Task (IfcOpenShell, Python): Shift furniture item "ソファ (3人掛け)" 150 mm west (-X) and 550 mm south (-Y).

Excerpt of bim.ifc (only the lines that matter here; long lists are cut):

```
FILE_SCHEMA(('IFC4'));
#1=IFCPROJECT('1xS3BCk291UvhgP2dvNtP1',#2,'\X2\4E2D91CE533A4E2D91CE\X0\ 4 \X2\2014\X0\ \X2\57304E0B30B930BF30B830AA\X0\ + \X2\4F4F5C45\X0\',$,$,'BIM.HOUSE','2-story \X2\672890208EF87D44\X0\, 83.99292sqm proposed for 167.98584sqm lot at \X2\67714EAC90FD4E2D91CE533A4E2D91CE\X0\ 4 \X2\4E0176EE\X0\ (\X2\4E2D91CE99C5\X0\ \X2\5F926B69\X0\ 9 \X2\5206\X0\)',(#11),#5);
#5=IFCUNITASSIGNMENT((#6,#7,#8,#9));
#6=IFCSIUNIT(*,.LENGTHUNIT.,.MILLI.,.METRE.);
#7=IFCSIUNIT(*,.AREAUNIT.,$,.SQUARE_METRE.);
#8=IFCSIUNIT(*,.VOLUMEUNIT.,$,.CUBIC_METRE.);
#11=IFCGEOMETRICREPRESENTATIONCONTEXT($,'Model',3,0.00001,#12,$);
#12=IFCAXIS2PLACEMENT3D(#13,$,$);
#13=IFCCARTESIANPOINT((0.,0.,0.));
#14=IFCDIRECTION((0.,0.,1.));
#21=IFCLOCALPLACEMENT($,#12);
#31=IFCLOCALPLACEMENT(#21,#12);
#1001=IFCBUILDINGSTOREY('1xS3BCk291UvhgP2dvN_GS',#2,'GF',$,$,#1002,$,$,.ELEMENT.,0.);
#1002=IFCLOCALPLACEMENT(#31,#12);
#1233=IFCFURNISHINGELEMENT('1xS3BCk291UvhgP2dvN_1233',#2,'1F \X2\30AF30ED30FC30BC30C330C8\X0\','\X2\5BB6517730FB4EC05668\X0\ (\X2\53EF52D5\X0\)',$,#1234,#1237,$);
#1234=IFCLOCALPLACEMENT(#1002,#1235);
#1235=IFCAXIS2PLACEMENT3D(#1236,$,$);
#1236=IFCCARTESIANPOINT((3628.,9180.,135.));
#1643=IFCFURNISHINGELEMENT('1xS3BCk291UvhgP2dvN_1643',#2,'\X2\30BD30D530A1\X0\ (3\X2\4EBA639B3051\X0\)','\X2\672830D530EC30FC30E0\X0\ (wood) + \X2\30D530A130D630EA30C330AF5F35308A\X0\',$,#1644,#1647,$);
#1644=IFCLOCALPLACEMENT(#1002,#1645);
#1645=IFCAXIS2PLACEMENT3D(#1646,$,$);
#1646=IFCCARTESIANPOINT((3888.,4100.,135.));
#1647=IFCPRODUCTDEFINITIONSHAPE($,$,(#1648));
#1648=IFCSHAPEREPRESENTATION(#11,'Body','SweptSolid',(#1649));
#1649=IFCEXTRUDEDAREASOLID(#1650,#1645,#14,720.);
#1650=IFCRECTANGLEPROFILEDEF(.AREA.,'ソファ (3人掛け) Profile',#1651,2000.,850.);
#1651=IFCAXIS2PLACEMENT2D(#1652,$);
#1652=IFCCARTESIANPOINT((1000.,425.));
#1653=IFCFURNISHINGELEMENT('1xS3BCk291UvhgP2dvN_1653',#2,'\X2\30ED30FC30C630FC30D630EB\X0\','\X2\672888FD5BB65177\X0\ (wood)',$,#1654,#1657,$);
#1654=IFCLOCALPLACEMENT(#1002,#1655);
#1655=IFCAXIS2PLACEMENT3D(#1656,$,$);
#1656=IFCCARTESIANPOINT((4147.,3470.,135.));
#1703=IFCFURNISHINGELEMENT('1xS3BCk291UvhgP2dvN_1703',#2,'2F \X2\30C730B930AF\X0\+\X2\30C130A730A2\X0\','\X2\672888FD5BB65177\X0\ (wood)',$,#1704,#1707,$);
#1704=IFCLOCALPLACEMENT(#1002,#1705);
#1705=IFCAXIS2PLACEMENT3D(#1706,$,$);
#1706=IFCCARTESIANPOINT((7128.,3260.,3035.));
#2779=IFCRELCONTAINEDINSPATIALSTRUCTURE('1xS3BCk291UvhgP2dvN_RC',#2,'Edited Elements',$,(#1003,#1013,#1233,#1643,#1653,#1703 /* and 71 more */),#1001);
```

```python
import ifcopenshell
import ifcopenshell.api.geometry
import ifcopenshell.util.placement
import ifcopenshell.util.unit

model = ifcopenshell.open("bim.ifc")
unit_scale = ifcopenshell.util.unit.calculate_unit_scale(model)

item = model.by_id(1643)
matrix = ifcopenshell.util.placement.get_local_placement(item.ObjectPlacement)
matrix[0, 3] -= 0.15 / unit_scale
matrix[1, 3] -= 0.55 / unit_scale
ifcopenshell.api.geometry.edit_object_placement(model, product=item, matrix=matrix, is_si=False)

print(ifcopenshell.util.placement.get_local_placement(item.ObjectPlacement).round(3) + 0.0)

model.write("bim_v2.ifc")
```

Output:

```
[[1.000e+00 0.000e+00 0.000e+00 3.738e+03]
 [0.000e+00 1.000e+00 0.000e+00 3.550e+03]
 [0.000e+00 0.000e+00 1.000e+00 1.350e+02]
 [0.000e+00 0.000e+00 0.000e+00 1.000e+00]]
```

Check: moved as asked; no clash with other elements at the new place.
